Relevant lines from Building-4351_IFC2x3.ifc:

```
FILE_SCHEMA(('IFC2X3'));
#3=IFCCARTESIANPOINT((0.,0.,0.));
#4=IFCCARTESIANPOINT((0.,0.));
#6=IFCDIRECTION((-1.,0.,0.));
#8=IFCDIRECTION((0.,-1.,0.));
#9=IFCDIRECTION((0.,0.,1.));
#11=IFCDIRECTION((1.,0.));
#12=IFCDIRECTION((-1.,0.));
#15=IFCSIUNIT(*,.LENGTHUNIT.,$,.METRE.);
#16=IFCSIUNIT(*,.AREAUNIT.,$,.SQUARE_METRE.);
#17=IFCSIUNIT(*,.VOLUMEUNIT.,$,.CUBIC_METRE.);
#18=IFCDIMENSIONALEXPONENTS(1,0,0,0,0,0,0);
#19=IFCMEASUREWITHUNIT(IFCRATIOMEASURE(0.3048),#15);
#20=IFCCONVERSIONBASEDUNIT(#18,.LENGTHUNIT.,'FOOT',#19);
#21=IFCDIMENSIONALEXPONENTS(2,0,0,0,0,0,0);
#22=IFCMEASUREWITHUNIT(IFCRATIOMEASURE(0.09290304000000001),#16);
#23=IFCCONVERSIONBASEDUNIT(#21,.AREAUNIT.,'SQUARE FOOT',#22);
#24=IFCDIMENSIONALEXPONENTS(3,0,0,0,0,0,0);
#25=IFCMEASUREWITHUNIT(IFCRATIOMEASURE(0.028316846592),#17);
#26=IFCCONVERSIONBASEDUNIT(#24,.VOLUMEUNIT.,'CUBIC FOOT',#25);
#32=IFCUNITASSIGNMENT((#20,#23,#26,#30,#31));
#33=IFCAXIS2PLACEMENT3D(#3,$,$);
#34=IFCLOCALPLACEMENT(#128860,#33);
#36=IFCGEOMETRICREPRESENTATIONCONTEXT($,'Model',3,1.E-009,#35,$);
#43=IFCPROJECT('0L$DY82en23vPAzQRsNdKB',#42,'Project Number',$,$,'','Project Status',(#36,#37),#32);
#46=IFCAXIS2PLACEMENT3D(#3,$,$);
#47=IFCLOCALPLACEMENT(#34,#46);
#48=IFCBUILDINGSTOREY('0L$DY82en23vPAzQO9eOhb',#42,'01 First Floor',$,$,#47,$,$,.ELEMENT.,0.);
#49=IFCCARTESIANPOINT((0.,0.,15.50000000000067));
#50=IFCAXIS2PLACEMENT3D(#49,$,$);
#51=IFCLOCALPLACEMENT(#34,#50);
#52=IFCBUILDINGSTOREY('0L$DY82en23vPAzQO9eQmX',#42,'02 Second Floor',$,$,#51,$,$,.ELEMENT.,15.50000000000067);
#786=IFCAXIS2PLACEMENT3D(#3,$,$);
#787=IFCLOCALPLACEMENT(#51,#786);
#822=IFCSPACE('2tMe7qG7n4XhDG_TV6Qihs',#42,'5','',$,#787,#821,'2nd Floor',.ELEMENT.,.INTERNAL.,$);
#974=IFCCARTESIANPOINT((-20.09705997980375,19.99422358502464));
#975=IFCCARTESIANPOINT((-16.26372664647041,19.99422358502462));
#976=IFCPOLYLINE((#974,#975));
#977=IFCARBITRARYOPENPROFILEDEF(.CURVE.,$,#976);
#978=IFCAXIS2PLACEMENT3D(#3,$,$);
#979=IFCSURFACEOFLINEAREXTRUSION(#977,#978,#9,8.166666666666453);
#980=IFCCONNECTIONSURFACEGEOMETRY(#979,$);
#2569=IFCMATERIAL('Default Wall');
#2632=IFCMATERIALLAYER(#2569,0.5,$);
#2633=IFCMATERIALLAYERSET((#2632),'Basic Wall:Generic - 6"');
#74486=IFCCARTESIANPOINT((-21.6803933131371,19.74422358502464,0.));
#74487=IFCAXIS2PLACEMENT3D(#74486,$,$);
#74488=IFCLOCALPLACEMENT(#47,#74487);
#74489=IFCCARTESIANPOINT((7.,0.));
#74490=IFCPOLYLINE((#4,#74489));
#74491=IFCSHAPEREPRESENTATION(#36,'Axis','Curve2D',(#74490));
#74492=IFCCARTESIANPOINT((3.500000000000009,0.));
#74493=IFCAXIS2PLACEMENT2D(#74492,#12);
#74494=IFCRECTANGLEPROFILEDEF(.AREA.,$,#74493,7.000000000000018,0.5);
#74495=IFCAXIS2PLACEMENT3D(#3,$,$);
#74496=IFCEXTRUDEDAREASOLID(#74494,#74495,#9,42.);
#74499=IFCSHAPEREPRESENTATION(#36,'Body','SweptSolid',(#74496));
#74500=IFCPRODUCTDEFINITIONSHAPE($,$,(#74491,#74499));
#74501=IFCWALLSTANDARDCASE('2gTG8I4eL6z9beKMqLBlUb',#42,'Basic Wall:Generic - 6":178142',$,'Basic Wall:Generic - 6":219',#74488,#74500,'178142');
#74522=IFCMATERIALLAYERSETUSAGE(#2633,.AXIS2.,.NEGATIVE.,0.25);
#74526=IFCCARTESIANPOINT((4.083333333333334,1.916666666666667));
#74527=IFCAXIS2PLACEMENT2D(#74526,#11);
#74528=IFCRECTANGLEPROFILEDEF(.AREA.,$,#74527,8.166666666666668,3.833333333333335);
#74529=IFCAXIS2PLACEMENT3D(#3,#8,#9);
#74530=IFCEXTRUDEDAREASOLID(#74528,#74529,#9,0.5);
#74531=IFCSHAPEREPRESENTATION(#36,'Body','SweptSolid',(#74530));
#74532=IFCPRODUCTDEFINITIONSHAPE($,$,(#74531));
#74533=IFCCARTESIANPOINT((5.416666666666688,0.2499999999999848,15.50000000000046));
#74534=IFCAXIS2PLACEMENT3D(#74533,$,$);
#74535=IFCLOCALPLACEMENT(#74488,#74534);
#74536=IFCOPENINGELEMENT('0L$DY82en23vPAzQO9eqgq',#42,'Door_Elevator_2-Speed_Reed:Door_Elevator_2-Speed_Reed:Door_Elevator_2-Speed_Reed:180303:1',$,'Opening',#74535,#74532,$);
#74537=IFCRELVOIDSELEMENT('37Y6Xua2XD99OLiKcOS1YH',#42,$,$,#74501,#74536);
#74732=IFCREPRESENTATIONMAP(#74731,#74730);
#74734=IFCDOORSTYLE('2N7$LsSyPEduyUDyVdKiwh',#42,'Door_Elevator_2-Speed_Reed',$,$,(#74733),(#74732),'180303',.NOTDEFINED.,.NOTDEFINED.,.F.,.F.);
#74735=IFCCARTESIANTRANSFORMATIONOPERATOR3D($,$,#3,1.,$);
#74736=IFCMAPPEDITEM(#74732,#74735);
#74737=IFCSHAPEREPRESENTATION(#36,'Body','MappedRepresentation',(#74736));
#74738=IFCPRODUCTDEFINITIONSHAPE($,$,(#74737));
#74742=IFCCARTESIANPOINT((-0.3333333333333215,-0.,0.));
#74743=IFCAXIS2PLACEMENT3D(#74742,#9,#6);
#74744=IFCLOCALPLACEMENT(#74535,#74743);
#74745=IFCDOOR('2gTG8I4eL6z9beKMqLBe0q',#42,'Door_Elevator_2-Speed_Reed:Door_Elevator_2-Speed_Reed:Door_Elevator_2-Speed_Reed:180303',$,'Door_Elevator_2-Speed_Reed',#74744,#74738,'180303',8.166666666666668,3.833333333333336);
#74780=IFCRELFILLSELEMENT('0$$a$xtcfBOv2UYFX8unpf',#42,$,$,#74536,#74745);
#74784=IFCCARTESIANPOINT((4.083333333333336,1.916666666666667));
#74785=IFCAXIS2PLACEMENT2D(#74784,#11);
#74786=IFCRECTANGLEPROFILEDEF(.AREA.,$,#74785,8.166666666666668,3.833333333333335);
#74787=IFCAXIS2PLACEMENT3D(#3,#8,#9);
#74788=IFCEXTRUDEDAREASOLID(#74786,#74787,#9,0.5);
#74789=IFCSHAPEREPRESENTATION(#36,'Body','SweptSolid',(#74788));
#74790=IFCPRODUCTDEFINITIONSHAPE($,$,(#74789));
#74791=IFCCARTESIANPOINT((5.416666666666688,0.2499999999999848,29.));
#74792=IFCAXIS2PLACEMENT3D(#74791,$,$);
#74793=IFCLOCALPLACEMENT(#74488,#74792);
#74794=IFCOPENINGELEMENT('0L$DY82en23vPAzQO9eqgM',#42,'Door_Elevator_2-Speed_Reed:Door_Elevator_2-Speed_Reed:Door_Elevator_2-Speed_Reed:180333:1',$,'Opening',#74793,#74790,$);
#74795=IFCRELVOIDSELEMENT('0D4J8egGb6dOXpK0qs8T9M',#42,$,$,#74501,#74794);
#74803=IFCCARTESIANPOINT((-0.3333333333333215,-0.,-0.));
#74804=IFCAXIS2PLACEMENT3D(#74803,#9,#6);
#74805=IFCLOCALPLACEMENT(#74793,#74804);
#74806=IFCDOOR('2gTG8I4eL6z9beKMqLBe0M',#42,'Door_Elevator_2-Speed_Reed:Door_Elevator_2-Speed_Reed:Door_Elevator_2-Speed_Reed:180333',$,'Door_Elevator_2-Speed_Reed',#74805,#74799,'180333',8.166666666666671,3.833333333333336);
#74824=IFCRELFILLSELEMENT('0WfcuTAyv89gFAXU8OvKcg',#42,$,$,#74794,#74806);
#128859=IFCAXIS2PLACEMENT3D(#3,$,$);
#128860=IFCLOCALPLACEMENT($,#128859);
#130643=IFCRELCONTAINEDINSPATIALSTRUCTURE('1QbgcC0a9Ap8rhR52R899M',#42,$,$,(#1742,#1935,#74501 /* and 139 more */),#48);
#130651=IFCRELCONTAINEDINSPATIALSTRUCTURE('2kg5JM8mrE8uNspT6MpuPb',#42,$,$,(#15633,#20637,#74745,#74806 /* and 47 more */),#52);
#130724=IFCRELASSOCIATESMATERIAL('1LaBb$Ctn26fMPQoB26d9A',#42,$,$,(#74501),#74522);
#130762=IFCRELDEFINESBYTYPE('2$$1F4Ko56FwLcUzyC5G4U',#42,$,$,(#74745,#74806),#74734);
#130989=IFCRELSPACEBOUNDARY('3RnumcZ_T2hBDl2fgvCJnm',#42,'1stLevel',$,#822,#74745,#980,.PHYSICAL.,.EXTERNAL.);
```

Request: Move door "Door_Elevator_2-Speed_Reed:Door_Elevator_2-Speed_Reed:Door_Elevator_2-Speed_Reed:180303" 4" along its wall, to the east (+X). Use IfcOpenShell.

```python
import numpy as np
import ifcopenshell
import ifcopenshell.api.geometry
import ifcopenshell.util.placement
import ifcopenshell.util.unit

model = ifcopenshell.open("Building-4351_IFC2x3.ifc")
unit_scale = ifcopenshell.util.unit.calculate_unit_scale(model)

door = model.by_guid("2gTG8I4eL6z9beKMqLBe0q")
opening = door.FillsVoids[0].RelatingOpeningElement
wall = opening.VoidsElements[0].RelatingBuildingElement

wall_matrix = ifcopenshell.util.placement.get_local_placement(wall.ObjectPlacement)
shift = wall_matrix[:3, 0] * 4 * 0.0254 / unit_scale
before = ifcopenshell.util.placement.get_local_placement(door.ObjectPlacement)[:3, 3].copy()

# The door is placed relative to its opening, so it follows when the opening moves.
matrix = ifcopenshell.util.placement.get_local_placement(opening.ObjectPlacement)
matrix[:3, 3] += shift
ifcopenshell.api.geometry.edit_object_placement(
    model, product=opening, matrix=matrix, is_si=False, should_transform_children=True
)

# Space boundary surfaces are stored in each space's coordinates; move them too.
for rel in door.ProvidesBoundaries:
    if not rel.ConnectionGeometry:
        continue
    surface = rel.ConnectionGeometry.SurfaceOnRelatingElement
    space_matrix = ifcopenshell.util.placement.get_local_placement(rel.RelatingSpace.ObjectPlacement)
    point = np.array(surface.Position.Location.Coordinates) + space_matrix[:3, :3].T @ shift
    surface.Position = model.createIfcAxis2Placement3D(
        model.createIfcCartesianPoint(point.tolist()), surface.Position.Axis, surface.Position.RefDirection
    )

after = ifcopenshell.util.placement.get_local_placement(door.ObjectPlacement)[:3, 3]
print("door moved by", (after - before).round(3) + 0.0)

model.write("Building-4351_IFC2x3_rev.ifc")
```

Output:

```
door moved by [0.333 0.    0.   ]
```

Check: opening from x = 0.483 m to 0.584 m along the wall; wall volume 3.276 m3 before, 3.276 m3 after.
